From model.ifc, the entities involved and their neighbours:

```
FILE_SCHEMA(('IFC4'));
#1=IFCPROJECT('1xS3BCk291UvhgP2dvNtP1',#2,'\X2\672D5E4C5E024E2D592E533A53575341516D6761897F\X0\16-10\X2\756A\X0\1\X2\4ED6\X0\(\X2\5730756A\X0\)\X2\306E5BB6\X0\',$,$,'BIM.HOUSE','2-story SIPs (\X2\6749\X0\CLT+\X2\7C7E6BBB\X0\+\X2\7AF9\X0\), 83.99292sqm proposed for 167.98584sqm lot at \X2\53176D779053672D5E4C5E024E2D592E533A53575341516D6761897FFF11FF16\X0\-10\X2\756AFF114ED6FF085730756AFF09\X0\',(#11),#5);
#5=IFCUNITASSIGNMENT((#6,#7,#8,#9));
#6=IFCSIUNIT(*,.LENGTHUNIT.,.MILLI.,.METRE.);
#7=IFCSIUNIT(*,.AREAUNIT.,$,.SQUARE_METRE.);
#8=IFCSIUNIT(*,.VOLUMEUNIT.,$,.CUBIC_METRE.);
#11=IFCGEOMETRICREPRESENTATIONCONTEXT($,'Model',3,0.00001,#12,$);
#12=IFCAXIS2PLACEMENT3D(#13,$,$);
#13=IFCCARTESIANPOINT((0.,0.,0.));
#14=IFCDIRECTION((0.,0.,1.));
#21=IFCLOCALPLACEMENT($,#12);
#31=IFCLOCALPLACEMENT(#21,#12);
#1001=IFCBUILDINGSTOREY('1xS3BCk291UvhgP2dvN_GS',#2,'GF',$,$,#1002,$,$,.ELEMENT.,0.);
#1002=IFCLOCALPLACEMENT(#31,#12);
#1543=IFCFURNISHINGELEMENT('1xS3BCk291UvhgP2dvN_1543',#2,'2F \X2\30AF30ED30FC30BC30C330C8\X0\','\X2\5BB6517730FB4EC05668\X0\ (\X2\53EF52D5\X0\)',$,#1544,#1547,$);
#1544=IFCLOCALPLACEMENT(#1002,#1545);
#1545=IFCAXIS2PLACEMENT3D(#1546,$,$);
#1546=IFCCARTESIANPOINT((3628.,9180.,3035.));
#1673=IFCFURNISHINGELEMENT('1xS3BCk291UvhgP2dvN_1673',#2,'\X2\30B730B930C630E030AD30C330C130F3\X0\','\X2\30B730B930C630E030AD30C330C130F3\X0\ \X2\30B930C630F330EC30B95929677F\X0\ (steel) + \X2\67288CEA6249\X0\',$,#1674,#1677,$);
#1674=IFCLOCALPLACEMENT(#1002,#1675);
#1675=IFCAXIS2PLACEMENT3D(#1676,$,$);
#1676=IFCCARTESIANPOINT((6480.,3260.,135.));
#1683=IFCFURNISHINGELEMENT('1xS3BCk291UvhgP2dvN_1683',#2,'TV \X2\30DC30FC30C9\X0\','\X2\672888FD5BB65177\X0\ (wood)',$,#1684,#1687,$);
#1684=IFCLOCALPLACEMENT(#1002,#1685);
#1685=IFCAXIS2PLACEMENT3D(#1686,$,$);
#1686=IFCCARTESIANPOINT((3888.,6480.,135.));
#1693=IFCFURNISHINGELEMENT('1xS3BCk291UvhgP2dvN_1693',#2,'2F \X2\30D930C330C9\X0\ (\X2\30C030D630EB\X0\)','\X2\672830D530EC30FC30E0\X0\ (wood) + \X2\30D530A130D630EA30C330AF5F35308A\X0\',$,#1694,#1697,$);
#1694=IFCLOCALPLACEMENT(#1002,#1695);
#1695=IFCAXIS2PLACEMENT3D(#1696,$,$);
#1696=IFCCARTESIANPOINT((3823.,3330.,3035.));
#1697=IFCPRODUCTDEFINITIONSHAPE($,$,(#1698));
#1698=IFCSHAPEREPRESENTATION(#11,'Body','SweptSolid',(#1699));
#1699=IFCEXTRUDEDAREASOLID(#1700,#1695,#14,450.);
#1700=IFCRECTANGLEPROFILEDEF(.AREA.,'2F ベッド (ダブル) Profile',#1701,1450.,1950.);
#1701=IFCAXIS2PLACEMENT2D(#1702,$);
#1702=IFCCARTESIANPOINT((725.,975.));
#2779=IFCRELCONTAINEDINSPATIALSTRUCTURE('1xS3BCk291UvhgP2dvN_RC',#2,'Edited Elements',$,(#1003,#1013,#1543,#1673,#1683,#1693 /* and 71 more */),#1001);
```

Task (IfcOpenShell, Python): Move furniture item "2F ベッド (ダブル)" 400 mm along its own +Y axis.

```python
import ifcopenshell
import ifcopenshell.api.geometry
import ifcopenshell.util.placement
import ifcopenshell.util.unit

model = ifcopenshell.open("model.ifc")
unit_scale = ifcopenshell.util.unit.calculate_unit_scale(model)

item = model.by_id(1693)
matrix = ifcopenshell.util.placement.get_local_placement(item.ObjectPlacement)
matrix[:3, 3] += matrix[:3, 1] * 0.4 / unit_scale
ifcopenshell.api.geometry.edit_object_placement(model, product=item, matrix=matrix, is_si=False)

print(ifcopenshell.util.placement.get_local_placement(item.ObjectPlacement).round(3) + 0.0)

model.write("model_rev.ifc")
```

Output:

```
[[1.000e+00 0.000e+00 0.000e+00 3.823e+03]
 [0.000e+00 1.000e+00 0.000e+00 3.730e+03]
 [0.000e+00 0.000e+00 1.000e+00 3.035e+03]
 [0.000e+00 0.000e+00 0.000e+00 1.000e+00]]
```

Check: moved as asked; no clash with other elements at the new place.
